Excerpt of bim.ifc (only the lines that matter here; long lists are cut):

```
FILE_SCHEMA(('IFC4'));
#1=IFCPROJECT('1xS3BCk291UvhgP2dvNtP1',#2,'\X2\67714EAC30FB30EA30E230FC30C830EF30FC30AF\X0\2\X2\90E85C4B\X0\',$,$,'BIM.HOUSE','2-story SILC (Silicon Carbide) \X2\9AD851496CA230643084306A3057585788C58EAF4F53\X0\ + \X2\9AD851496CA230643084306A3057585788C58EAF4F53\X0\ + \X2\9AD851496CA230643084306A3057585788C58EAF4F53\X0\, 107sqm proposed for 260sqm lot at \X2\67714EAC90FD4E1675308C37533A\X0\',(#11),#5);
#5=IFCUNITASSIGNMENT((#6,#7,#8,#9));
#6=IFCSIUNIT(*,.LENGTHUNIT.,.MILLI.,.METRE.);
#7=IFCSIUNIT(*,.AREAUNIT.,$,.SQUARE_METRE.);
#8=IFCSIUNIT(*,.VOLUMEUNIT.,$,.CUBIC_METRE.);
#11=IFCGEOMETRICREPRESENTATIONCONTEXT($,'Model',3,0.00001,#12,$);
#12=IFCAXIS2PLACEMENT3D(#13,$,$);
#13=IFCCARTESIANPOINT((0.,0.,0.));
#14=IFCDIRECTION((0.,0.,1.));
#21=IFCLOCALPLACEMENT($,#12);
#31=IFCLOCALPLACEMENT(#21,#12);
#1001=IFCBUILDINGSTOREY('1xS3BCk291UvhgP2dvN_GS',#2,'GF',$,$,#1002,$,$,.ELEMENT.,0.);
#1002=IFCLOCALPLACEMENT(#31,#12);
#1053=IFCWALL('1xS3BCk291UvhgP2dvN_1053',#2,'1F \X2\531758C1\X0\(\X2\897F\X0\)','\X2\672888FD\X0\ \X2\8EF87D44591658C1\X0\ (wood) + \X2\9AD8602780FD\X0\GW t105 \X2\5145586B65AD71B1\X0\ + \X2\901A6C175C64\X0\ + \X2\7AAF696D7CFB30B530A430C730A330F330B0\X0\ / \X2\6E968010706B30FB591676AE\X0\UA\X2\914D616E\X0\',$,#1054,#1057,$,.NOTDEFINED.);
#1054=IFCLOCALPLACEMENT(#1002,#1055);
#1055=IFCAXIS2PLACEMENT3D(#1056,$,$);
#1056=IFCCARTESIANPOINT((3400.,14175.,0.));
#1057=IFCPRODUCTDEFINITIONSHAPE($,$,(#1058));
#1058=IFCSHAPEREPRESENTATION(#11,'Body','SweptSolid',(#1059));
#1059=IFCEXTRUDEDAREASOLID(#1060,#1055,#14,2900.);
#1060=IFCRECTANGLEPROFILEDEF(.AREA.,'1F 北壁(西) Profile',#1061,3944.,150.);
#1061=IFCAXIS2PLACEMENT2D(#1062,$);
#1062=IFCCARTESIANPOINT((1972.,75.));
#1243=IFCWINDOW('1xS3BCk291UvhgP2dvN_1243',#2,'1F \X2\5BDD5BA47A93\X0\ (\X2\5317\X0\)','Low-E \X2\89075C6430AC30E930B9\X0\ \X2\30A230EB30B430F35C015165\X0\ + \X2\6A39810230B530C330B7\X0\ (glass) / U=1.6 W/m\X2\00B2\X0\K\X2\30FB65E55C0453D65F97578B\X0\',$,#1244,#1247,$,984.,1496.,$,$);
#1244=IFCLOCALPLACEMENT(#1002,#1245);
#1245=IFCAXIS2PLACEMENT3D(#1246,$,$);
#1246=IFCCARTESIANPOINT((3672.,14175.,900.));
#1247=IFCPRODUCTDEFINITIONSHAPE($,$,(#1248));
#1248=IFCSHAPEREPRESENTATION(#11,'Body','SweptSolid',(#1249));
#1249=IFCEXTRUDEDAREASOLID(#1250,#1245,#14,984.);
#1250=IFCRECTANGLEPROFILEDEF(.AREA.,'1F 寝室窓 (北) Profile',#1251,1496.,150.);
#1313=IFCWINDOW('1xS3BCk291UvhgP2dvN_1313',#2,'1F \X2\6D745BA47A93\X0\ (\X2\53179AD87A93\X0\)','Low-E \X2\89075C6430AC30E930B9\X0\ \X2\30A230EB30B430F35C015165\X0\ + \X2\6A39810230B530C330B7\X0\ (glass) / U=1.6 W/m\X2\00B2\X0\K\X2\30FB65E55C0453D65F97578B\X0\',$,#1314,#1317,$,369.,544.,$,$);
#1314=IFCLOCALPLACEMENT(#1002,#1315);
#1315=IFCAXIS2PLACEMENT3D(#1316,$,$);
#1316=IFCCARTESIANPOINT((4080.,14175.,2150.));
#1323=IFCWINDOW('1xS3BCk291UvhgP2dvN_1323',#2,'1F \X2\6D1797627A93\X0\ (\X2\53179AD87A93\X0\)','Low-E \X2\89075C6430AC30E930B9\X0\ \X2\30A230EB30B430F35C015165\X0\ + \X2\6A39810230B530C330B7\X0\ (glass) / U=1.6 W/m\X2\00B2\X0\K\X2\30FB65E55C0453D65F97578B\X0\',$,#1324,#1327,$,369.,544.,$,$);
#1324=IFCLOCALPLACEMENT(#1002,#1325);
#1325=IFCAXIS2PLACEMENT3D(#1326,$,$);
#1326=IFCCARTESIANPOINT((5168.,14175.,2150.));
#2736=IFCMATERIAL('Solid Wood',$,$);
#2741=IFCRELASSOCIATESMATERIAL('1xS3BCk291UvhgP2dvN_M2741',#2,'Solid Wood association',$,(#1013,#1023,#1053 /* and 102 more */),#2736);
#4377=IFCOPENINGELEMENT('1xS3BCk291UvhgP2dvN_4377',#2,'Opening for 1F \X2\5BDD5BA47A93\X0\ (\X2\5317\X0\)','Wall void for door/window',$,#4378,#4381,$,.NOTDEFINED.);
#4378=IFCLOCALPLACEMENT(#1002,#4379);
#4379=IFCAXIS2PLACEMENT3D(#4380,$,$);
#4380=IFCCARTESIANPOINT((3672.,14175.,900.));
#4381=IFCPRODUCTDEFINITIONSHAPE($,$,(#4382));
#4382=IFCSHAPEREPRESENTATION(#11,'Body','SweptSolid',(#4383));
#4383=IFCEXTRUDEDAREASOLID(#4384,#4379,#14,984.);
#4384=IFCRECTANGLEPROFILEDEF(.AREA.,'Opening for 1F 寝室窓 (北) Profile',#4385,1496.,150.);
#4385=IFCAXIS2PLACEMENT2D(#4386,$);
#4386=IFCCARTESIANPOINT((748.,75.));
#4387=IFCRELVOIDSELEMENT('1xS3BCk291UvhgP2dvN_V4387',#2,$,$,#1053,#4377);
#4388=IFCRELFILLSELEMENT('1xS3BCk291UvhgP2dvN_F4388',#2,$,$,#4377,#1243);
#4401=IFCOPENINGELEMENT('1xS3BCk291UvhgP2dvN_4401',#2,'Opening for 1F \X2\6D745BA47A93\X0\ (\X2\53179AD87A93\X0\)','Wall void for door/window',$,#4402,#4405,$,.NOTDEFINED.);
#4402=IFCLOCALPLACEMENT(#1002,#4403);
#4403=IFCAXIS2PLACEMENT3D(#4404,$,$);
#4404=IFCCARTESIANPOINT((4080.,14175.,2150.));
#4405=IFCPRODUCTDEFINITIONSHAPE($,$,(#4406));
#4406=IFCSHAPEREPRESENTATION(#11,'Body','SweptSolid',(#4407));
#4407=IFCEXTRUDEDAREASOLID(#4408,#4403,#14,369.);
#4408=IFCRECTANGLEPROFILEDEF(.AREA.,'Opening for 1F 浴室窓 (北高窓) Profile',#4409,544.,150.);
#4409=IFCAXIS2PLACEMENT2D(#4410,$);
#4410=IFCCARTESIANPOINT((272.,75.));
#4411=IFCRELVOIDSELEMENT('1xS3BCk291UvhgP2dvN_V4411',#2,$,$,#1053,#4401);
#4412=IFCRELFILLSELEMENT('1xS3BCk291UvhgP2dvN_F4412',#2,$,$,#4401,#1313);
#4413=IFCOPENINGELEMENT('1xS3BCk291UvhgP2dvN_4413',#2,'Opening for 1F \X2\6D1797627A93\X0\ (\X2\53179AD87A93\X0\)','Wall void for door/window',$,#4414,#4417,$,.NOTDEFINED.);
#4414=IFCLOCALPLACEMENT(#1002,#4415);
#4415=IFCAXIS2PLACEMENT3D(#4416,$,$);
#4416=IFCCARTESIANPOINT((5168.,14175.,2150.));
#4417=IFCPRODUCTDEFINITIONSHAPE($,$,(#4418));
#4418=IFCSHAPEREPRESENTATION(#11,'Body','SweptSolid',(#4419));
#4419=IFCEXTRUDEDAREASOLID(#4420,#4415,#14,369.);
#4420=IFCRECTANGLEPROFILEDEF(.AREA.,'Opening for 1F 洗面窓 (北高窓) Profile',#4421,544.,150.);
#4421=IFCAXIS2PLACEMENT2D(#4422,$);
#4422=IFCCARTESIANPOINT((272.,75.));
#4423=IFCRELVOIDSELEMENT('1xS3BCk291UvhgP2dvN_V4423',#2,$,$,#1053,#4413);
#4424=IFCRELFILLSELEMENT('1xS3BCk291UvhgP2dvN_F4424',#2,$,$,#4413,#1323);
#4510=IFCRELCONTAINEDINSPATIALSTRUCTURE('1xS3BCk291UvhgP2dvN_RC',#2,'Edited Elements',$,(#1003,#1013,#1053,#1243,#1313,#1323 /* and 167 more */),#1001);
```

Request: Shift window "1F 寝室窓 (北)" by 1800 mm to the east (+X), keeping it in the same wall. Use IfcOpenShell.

```python
import ifcopenshell
import ifcopenshell.api.geometry
import ifcopenshell.util.placement
import ifcopenshell.util.unit

model = ifcopenshell.open("bim.ifc")
unit_scale = ifcopenshell.util.unit.calculate_unit_scale(model)

window = model.by_guid("1xS3BCk291UvhgP2dvN_1243")
opening = window.FillsVoids[0].RelatingOpeningElement
wall = opening.VoidsElements[0].RelatingBuildingElement

wall_matrix = ifcopenshell.util.placement.get_local_placement(wall.ObjectPlacement)
shift = wall_matrix[:3, 0] * 1.8 / unit_scale
before = ifcopenshell.util.placement.get_local_placement(window.ObjectPlacement)[:3, 3].copy()

# The window is not placed relative to its opening, so move both.
for product in (opening, window):
    matrix = ifcopenshell.util.placement.get_local_placement(product.ObjectPlacement)
    matrix[:3, 3] += shift
    ifcopenshell.api.geometry.edit_object_placement(model, product=product, matrix=matrix, is_si=False)

after = ifcopenshell.util.placement.get_local_placement(window.ObjectPlacement)[:3, 3]
print("window moved by", (after - before).round(3) + 0.0)

model.write("bim_v2.ifc")
```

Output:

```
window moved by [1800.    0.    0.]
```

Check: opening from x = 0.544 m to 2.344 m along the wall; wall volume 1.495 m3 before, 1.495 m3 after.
